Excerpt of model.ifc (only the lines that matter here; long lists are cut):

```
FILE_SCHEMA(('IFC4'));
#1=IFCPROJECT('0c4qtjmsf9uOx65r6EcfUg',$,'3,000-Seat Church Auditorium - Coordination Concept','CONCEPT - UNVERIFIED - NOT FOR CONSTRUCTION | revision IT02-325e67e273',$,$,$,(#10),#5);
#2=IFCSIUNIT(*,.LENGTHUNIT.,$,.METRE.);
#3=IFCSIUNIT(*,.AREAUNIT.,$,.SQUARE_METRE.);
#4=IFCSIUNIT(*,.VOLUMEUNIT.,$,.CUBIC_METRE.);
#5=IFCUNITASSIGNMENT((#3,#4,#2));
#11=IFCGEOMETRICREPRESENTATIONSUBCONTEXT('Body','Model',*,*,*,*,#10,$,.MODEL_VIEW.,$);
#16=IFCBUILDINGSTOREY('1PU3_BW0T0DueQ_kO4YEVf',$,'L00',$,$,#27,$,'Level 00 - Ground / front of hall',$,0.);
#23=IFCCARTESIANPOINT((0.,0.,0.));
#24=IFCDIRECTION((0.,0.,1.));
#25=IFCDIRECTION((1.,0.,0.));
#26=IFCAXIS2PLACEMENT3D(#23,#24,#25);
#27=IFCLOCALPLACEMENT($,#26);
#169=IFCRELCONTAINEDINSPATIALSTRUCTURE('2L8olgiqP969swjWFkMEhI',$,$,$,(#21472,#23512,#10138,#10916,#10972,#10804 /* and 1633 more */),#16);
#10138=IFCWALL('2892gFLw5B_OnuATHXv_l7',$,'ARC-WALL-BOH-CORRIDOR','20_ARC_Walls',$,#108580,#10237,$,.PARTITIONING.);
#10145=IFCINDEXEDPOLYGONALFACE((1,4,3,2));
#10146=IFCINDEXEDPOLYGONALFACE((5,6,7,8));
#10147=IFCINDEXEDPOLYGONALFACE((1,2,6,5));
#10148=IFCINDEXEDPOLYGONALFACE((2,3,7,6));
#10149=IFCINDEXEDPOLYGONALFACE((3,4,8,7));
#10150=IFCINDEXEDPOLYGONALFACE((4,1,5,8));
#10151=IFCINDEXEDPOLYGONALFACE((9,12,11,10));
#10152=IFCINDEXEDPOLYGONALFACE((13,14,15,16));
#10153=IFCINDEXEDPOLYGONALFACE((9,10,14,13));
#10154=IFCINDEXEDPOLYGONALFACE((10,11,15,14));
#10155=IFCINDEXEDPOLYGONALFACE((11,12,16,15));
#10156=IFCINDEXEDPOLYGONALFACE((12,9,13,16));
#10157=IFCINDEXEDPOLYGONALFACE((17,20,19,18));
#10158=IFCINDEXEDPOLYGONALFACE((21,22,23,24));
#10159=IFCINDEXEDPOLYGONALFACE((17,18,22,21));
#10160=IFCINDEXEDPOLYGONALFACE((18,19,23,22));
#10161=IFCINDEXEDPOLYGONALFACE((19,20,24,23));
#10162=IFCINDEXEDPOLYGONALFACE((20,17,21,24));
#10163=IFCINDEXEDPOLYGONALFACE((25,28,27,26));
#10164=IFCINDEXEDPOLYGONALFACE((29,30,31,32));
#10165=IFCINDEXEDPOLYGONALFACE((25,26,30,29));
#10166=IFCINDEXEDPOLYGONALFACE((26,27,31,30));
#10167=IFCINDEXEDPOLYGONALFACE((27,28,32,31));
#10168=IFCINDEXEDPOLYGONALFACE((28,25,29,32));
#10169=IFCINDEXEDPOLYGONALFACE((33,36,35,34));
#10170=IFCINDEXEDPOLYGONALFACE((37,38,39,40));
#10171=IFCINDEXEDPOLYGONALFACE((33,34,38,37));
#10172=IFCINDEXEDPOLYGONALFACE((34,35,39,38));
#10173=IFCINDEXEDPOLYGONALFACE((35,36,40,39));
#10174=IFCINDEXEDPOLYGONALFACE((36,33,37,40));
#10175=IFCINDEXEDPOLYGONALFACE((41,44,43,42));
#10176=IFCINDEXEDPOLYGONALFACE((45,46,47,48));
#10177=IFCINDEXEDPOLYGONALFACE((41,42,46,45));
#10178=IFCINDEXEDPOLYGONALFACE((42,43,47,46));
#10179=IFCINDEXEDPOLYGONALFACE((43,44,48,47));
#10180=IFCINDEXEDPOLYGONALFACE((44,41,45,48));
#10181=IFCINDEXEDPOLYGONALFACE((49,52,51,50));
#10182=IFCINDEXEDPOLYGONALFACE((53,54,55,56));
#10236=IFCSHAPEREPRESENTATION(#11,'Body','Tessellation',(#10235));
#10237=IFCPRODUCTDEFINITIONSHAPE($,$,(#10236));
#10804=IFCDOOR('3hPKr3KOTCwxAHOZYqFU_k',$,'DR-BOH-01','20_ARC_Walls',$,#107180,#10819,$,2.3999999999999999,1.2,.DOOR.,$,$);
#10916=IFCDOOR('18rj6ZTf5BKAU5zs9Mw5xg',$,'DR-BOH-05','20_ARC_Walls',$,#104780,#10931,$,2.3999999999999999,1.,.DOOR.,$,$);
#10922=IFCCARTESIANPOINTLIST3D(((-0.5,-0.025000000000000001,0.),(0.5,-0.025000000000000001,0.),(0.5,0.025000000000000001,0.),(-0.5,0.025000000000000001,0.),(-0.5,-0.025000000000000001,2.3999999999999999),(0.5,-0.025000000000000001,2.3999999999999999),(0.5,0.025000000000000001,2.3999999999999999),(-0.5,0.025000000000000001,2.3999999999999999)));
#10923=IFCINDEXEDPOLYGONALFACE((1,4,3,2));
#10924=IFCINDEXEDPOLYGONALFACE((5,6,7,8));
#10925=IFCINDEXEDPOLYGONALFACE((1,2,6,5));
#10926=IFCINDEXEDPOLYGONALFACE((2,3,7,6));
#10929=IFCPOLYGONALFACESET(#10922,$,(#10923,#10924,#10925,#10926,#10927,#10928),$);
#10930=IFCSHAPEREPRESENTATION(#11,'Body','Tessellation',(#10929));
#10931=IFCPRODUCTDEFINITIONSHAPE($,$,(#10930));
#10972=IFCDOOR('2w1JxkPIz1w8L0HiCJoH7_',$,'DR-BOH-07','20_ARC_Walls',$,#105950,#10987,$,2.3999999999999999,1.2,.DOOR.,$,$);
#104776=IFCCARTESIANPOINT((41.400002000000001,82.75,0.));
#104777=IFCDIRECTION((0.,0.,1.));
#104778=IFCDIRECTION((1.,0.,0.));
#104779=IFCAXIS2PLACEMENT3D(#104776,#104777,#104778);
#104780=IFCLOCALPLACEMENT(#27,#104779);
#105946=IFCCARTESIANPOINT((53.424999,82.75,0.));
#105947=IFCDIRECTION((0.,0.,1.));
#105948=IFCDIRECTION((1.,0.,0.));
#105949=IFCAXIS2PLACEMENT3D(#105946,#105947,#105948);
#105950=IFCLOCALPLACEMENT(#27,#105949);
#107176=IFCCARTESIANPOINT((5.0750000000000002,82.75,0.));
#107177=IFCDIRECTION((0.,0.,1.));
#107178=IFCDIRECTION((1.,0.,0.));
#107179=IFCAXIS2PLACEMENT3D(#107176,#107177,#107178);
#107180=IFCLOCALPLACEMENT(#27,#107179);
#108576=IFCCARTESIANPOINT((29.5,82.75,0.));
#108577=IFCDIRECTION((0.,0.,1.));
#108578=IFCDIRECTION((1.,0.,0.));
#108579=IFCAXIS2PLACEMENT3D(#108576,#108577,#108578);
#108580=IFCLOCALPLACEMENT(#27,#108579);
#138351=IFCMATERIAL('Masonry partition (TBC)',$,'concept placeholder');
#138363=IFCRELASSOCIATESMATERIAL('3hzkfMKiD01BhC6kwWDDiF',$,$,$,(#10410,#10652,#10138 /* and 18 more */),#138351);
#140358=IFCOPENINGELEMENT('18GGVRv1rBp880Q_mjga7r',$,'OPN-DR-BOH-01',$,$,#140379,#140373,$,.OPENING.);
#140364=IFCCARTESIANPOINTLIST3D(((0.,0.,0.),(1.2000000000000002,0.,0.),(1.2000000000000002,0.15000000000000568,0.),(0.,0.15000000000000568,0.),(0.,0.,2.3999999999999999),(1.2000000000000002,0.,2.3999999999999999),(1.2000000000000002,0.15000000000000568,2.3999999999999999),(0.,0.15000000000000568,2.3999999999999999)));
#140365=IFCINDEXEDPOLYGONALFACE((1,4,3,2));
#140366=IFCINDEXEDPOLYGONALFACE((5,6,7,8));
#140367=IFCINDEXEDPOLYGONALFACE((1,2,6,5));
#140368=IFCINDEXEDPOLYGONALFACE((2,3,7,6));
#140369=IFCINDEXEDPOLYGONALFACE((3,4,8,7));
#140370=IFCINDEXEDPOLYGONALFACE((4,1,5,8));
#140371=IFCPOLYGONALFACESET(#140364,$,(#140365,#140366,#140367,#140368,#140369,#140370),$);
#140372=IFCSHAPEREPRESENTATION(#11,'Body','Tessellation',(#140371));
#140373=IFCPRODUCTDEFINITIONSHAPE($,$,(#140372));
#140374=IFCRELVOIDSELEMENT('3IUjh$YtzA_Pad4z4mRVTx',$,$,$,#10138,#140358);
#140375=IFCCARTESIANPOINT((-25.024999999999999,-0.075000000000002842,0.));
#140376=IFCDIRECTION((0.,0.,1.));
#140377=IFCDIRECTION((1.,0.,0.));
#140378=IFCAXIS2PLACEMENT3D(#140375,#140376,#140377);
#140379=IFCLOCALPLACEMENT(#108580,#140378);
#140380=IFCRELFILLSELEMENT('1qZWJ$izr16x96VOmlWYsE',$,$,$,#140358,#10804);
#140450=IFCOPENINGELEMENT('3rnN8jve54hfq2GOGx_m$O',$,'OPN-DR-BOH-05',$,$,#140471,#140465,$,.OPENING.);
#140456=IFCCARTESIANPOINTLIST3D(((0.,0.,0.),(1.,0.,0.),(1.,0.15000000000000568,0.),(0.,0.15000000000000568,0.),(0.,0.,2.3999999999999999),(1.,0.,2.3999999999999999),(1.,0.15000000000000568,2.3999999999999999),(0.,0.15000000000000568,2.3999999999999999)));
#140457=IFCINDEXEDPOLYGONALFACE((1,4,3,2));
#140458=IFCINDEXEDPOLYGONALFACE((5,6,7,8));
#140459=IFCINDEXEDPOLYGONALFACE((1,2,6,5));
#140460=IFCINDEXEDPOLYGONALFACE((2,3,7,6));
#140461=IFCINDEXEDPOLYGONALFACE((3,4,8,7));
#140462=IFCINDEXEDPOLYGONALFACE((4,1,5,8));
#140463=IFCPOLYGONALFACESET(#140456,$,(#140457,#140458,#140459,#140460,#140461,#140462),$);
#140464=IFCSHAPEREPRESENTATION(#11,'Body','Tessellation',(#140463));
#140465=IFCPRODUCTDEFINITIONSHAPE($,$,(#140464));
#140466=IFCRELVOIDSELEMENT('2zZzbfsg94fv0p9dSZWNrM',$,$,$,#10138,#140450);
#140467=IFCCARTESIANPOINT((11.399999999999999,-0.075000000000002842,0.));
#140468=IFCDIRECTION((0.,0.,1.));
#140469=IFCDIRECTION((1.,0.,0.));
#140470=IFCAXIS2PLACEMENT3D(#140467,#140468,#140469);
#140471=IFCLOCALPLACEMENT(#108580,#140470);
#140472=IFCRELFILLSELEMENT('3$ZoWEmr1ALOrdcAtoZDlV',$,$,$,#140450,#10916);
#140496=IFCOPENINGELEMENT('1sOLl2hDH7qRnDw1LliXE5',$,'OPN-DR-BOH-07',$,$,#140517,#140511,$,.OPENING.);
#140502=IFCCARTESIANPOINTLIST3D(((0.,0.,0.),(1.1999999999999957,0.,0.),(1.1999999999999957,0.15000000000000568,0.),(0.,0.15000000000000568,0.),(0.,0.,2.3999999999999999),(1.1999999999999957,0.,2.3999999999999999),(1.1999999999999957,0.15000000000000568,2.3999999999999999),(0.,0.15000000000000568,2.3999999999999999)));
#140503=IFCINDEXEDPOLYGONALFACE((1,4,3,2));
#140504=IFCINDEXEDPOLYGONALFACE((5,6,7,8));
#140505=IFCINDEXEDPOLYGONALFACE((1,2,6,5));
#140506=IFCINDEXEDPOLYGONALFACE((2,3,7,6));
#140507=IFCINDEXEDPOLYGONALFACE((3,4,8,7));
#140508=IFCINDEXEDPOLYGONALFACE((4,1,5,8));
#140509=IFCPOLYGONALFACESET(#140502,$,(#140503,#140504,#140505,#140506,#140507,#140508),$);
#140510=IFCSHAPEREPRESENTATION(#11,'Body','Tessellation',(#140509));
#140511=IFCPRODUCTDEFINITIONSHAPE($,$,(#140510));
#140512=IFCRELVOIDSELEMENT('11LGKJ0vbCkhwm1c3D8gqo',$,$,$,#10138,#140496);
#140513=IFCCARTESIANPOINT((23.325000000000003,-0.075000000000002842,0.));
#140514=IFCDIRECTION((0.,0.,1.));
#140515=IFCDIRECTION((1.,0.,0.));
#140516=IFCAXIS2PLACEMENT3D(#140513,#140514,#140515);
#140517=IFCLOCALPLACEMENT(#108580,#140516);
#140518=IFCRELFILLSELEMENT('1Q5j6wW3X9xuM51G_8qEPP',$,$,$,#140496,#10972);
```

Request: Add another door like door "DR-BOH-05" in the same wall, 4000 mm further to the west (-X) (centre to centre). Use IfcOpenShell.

```python
import ifcopenshell
import ifcopenshell.api.feature
import ifcopenshell.api.geometry
import ifcopenshell.api.root
import ifcopenshell.geom
import ifcopenshell.util.element
import ifcopenshell.util.placement
import ifcopenshell.util.shape
import ifcopenshell.util.unit

model = ifcopenshell.open("model.ifc")
unit_scale = ifcopenshell.util.unit.calculate_unit_scale(model)
settings = ifcopenshell.geom.settings()


def volume(element):
    """Net volume in cubic metres, openings subtracted."""
    shape = ifcopenshell.geom.create_shape(settings, element)
    return ifcopenshell.util.shape.get_volume(shape.geometry)


door = model.by_guid("18rj6ZTf5BKAU5zs9Mw5xg")
opening = door.FillsVoids[0].RelatingOpeningElement
wall = opening.VoidsElements[0].RelatingBuildingElement
before = volume(wall)
shift = ifcopenshell.util.placement.get_local_placement(wall.ObjectPlacement)[:3, 0] * -4 / unit_scale

# copy_class copies the void relationship, type, container and properties, but no geometry.
new_opening = ifcopenshell.api.root.copy_class(model, product=opening)
new_opening.Representation = ifcopenshell.util.element.copy_deep(
    model, opening.Representation, exclude=["IfcGeometricRepresentationContext", "IfcRepresentationMap"]
)
new_door = ifcopenshell.api.root.copy_class(model, product=door)
new_door.Representation = ifcopenshell.util.element.copy_deep(
    model, door.Representation, exclude=["IfcGeometricRepresentationContext", "IfcRepresentationMap"]
)
ifcopenshell.api.feature.add_filling(model, opening=new_opening, element=new_door)

for old, new in ((opening, new_opening), (door, new_door)):
    matrix = ifcopenshell.util.placement.get_local_placement(old.ObjectPlacement)
    matrix[:3, 3] += shift
    ifcopenshell.api.geometry.edit_object_placement(model, product=new, matrix=matrix, is_si=False)

after = volume(wall)

print(f"wall volume {before:.3f} -> {after:.3f} m3")

model.write("model_edited.ifc")
```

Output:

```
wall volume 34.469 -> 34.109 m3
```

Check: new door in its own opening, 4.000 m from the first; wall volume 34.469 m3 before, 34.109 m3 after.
